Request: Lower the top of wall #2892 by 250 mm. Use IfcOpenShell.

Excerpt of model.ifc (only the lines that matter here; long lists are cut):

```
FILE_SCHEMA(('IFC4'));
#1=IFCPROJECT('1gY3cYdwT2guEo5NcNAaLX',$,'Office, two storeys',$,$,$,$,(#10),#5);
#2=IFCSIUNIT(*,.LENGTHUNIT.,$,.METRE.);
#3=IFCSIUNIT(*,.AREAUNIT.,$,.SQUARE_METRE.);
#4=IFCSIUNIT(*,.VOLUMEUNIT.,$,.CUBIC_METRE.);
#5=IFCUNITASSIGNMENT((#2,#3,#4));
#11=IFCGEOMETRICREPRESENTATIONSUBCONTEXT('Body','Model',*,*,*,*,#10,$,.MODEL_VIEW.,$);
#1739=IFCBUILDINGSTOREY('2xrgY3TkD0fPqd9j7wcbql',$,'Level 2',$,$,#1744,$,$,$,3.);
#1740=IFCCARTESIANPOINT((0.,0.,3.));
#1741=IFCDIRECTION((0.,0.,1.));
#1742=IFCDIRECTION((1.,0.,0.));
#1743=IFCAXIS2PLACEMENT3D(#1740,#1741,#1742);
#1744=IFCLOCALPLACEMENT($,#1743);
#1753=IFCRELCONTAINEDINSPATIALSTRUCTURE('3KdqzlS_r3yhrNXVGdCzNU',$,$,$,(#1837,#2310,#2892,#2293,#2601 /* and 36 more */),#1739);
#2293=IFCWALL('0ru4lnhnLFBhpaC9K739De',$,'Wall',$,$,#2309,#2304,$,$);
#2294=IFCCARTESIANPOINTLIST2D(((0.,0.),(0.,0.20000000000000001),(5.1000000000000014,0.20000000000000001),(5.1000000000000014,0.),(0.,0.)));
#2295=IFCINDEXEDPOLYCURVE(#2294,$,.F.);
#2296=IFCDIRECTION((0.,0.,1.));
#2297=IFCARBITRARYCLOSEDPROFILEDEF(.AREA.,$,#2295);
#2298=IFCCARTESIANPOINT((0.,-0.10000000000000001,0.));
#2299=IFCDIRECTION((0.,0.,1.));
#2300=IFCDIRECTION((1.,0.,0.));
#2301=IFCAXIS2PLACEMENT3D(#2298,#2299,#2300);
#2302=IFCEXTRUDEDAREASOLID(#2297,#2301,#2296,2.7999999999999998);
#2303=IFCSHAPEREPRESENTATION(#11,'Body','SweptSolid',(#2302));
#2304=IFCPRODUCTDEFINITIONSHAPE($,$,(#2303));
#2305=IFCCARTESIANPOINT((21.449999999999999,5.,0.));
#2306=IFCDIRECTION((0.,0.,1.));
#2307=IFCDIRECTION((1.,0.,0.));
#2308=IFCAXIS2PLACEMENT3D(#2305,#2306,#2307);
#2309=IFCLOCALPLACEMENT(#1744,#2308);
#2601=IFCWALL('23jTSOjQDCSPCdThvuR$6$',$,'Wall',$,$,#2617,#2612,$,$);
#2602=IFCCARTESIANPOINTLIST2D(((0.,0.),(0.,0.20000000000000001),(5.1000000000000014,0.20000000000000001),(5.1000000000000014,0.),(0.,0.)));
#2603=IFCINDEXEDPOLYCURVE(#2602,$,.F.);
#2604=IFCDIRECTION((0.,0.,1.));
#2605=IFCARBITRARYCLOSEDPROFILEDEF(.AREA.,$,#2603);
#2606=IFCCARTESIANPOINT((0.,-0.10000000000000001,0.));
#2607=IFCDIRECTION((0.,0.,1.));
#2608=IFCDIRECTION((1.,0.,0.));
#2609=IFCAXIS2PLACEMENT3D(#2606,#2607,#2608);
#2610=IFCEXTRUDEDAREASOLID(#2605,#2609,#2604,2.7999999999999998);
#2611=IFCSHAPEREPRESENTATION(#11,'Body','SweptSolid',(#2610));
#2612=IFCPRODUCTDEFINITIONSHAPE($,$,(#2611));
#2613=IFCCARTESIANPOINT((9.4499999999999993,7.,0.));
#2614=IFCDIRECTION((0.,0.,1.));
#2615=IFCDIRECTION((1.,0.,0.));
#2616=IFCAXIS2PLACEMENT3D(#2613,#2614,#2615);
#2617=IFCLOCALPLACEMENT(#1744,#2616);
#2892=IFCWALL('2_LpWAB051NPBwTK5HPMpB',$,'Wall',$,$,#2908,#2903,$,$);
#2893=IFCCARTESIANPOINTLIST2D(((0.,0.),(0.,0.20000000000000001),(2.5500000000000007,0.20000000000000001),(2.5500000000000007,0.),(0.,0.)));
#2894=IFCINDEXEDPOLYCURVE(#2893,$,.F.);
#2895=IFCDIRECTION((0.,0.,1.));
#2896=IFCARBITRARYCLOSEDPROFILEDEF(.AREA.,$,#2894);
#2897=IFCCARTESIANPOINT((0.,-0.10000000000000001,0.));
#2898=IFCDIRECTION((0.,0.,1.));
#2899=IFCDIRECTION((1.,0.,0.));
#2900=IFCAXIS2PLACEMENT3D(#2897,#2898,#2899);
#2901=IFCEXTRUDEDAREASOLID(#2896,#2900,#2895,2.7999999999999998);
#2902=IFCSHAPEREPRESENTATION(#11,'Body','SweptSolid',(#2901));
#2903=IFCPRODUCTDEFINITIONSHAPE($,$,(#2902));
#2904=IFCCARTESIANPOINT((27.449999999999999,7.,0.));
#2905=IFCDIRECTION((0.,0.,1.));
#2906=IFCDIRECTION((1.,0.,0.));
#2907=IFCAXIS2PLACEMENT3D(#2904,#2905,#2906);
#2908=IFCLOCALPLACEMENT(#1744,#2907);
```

```python
import ifcopenshell
import ifcopenshell.geom
import ifcopenshell.util.representation
import ifcopenshell.util.shape
import ifcopenshell.util.unit

model = ifcopenshell.open("model.ifc")
unit_scale = ifcopenshell.util.unit.calculate_unit_scale(model)
settings = ifcopenshell.geom.settings()


def volume(element):
    """Net volume in cubic metres, openings subtracted."""
    shape = ifcopenshell.geom.create_shape(settings, element)
    return ifcopenshell.util.shape.get_volume(shape.geometry)


wall = model.by_guid("2_LpWAB051NPBwTK5HPMpB")
before = volume(wall)

body = ifcopenshell.util.representation.get_representation(wall, "Model", "Body")
solid = body.Items[0]
old_height = solid.Depth
solid.Depth -= 0.25 / unit_scale
after = volume(wall)

print(f"height {old_height:g} -> {solid.Depth:g}, volume {before:.3f} -> {after:.3f} m3")

model.write("model_v2.ifc")
```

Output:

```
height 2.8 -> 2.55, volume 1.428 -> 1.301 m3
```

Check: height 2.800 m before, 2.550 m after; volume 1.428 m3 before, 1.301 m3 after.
